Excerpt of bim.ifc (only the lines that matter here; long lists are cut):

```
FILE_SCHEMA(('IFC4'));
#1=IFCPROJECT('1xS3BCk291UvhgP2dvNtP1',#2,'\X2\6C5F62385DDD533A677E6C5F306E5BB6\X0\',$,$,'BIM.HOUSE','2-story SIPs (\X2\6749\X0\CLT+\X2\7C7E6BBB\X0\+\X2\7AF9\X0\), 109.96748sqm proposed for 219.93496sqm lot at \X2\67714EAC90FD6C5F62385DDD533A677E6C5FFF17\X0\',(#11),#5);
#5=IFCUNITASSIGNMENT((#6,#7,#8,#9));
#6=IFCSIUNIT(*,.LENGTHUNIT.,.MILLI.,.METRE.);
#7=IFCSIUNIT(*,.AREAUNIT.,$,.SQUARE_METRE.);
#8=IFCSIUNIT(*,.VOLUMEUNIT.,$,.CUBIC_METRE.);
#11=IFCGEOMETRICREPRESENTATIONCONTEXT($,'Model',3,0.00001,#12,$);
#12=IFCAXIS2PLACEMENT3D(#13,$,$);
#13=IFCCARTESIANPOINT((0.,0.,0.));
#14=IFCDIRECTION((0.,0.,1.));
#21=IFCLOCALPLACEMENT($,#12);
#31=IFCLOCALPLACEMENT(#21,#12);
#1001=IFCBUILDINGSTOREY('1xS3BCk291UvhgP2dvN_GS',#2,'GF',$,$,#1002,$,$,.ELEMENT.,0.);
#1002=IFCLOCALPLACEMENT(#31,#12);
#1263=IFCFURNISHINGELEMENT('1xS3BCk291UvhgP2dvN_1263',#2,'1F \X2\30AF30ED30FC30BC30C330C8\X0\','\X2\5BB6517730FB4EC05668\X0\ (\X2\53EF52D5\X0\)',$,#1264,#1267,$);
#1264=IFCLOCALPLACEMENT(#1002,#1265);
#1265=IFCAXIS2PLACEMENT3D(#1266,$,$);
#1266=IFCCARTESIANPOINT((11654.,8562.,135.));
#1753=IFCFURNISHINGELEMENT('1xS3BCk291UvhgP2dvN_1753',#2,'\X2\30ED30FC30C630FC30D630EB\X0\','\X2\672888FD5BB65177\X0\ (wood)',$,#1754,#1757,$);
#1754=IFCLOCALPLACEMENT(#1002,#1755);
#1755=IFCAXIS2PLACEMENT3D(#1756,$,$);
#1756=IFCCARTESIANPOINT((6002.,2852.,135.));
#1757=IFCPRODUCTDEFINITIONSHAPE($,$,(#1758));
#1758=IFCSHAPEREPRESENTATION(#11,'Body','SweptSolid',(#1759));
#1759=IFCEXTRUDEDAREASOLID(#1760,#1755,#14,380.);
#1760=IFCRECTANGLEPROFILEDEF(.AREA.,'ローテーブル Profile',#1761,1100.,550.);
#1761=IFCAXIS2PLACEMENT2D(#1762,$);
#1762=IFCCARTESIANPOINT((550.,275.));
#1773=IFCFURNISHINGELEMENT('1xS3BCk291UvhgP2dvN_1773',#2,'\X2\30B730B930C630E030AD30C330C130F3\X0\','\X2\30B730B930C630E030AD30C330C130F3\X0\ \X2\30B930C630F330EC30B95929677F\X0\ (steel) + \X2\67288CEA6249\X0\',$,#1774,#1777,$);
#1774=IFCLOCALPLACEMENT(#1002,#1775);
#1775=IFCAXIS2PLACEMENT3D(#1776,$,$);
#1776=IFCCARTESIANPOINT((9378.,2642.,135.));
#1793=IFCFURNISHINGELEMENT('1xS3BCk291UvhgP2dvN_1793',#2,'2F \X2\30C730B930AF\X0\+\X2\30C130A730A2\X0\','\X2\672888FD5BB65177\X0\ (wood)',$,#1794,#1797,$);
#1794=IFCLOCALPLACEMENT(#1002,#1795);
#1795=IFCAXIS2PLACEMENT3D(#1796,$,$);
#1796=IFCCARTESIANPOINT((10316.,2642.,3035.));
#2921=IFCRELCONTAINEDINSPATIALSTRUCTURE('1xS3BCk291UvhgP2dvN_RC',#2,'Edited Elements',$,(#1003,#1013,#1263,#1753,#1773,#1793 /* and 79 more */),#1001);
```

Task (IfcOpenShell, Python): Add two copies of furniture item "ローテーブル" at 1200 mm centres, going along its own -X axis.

```python
import ifcopenshell
import ifcopenshell.api.geometry
import ifcopenshell.api.root
import ifcopenshell.util.element
import ifcopenshell.util.placement
import ifcopenshell.util.unit

model = ifcopenshell.open("bim.ifc")
unit_scale = ifcopenshell.util.unit.calculate_unit_scale(model)


def reuse_history(source, copy):
    """copy_class also copies each property set's owner history, people and application; keep the originals."""
    for rel in copy.IsDefinedBy:
        if rel.is_a("IfcRelDefinesByProperties") and (history := rel.RelatingPropertyDefinition.OwnerHistory):
            rel.RelatingPropertyDefinition.OwnerHistory = source.OwnerHistory
            ifcopenshell.util.element.remove_deep2(model, history)


source = model.by_guid("1xS3BCk291UvhgP2dvN_1753")
base = ifcopenshell.util.placement.get_local_placement(source.ObjectPlacement)
step = -base[:3, 0] * 1.2 / unit_scale

for i in range(1, 3):
    copy = ifcopenshell.api.root.copy_class(model, product=source)
    copy.Representation = ifcopenshell.util.element.copy_deep(
        model, source.Representation, exclude=["IfcGeometricRepresentationContext", "IfcRepresentationMap"]
    )
    reuse_history(source, copy)
    matrix = base.copy()
    matrix[:3, 3] += i * step
    print("added at", matrix[:3, 3].round(3) + 0.0)
    ifcopenshell.api.geometry.edit_object_placement(model, product=copy, matrix=matrix, is_si=False)

model.write("bim_updated.ifc")
```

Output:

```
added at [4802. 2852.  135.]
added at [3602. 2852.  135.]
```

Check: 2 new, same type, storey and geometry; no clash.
